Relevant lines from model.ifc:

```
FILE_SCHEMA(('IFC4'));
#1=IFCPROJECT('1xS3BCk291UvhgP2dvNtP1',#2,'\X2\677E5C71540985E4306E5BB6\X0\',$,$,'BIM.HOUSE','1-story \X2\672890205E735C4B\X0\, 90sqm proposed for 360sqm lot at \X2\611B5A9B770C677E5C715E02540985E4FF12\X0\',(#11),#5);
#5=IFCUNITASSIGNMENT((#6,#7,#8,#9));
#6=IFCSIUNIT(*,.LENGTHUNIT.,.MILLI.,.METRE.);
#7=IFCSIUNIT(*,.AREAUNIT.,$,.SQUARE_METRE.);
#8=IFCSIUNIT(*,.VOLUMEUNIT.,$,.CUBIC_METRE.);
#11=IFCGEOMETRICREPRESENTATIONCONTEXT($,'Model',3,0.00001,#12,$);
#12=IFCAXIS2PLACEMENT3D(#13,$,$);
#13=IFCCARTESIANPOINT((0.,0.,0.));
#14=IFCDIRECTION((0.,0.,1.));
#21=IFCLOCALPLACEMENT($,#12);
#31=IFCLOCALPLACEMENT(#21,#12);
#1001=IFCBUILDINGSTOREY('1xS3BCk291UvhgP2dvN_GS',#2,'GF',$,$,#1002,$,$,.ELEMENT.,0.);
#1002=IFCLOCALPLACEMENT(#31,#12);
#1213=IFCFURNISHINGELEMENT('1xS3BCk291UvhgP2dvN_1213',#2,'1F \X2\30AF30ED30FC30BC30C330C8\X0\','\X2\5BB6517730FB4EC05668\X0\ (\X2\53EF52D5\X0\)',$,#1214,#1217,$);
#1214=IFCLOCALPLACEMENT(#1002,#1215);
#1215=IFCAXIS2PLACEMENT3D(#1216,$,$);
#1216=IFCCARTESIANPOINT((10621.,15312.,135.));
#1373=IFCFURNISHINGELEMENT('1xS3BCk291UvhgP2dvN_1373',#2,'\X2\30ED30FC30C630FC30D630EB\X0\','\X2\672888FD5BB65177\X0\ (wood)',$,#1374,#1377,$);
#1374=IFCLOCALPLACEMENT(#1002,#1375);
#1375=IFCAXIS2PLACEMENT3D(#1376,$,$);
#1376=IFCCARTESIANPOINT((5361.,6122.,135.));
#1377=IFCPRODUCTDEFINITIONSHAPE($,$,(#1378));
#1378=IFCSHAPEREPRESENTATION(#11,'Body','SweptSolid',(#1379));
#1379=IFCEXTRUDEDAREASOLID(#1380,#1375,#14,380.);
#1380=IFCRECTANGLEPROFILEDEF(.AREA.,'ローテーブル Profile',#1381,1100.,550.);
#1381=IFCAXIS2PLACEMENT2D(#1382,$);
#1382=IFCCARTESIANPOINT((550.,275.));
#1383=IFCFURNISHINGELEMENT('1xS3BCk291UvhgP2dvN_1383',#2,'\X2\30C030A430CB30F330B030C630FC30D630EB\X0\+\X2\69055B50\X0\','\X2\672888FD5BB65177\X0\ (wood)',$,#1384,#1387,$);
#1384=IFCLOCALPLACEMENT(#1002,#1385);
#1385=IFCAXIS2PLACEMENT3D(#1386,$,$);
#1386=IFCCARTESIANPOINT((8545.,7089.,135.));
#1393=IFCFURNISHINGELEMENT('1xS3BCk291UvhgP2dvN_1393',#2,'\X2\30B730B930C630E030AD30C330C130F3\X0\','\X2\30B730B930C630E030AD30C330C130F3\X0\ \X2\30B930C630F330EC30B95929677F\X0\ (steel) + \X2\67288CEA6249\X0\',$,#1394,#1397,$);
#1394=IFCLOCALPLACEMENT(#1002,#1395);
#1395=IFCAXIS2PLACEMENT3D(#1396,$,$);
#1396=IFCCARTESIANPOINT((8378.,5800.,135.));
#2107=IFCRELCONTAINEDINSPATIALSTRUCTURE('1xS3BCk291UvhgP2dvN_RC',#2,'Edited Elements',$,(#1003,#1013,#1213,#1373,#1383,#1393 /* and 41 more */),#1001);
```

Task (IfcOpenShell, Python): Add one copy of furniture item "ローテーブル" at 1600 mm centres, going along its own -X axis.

```python
import ifcopenshell
import ifcopenshell.api.geometry
import ifcopenshell.api.root
import ifcopenshell.util.element
import ifcopenshell.util.placement
import ifcopenshell.util.unit

model = ifcopenshell.open("model.ifc")
unit_scale = ifcopenshell.util.unit.calculate_unit_scale(model)


def reuse_history(source, copy):
    """copy_class also copies each property set's owner history, people and application; keep the originals."""
    for rel in copy.IsDefinedBy:
        if rel.is_a("IfcRelDefinesByProperties") and (history := rel.RelatingPropertyDefinition.OwnerHistory):
            rel.RelatingPropertyDefinition.OwnerHistory = source.OwnerHistory
            ifcopenshell.util.element.remove_deep2(model, history)


source = model.by_guid("1xS3BCk291UvhgP2dvN_1373")
base = ifcopenshell.util.placement.get_local_placement(source.ObjectPlacement)
step = -base[:3, 0] * 1.6 / unit_scale

for i in range(1, 2):
    copy = ifcopenshell.api.root.copy_class(model, product=source)
    copy.Representation = ifcopenshell.util.element.copy_deep(
        model, source.Representation, exclude=["IfcGeometricRepresentationContext", "IfcRepresentationMap"]
    )
    reuse_history(source, copy)
    matrix = base.copy()
    matrix[:3, 3] += i * step
    print("added at", matrix[:3, 3].round(3) + 0.0)
    ifcopenshell.api.geometry.edit_object_placement(model, product=copy, matrix=matrix, is_si=False)

model.write("model_updated.ifc")
```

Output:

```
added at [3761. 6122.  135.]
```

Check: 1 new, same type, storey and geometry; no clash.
